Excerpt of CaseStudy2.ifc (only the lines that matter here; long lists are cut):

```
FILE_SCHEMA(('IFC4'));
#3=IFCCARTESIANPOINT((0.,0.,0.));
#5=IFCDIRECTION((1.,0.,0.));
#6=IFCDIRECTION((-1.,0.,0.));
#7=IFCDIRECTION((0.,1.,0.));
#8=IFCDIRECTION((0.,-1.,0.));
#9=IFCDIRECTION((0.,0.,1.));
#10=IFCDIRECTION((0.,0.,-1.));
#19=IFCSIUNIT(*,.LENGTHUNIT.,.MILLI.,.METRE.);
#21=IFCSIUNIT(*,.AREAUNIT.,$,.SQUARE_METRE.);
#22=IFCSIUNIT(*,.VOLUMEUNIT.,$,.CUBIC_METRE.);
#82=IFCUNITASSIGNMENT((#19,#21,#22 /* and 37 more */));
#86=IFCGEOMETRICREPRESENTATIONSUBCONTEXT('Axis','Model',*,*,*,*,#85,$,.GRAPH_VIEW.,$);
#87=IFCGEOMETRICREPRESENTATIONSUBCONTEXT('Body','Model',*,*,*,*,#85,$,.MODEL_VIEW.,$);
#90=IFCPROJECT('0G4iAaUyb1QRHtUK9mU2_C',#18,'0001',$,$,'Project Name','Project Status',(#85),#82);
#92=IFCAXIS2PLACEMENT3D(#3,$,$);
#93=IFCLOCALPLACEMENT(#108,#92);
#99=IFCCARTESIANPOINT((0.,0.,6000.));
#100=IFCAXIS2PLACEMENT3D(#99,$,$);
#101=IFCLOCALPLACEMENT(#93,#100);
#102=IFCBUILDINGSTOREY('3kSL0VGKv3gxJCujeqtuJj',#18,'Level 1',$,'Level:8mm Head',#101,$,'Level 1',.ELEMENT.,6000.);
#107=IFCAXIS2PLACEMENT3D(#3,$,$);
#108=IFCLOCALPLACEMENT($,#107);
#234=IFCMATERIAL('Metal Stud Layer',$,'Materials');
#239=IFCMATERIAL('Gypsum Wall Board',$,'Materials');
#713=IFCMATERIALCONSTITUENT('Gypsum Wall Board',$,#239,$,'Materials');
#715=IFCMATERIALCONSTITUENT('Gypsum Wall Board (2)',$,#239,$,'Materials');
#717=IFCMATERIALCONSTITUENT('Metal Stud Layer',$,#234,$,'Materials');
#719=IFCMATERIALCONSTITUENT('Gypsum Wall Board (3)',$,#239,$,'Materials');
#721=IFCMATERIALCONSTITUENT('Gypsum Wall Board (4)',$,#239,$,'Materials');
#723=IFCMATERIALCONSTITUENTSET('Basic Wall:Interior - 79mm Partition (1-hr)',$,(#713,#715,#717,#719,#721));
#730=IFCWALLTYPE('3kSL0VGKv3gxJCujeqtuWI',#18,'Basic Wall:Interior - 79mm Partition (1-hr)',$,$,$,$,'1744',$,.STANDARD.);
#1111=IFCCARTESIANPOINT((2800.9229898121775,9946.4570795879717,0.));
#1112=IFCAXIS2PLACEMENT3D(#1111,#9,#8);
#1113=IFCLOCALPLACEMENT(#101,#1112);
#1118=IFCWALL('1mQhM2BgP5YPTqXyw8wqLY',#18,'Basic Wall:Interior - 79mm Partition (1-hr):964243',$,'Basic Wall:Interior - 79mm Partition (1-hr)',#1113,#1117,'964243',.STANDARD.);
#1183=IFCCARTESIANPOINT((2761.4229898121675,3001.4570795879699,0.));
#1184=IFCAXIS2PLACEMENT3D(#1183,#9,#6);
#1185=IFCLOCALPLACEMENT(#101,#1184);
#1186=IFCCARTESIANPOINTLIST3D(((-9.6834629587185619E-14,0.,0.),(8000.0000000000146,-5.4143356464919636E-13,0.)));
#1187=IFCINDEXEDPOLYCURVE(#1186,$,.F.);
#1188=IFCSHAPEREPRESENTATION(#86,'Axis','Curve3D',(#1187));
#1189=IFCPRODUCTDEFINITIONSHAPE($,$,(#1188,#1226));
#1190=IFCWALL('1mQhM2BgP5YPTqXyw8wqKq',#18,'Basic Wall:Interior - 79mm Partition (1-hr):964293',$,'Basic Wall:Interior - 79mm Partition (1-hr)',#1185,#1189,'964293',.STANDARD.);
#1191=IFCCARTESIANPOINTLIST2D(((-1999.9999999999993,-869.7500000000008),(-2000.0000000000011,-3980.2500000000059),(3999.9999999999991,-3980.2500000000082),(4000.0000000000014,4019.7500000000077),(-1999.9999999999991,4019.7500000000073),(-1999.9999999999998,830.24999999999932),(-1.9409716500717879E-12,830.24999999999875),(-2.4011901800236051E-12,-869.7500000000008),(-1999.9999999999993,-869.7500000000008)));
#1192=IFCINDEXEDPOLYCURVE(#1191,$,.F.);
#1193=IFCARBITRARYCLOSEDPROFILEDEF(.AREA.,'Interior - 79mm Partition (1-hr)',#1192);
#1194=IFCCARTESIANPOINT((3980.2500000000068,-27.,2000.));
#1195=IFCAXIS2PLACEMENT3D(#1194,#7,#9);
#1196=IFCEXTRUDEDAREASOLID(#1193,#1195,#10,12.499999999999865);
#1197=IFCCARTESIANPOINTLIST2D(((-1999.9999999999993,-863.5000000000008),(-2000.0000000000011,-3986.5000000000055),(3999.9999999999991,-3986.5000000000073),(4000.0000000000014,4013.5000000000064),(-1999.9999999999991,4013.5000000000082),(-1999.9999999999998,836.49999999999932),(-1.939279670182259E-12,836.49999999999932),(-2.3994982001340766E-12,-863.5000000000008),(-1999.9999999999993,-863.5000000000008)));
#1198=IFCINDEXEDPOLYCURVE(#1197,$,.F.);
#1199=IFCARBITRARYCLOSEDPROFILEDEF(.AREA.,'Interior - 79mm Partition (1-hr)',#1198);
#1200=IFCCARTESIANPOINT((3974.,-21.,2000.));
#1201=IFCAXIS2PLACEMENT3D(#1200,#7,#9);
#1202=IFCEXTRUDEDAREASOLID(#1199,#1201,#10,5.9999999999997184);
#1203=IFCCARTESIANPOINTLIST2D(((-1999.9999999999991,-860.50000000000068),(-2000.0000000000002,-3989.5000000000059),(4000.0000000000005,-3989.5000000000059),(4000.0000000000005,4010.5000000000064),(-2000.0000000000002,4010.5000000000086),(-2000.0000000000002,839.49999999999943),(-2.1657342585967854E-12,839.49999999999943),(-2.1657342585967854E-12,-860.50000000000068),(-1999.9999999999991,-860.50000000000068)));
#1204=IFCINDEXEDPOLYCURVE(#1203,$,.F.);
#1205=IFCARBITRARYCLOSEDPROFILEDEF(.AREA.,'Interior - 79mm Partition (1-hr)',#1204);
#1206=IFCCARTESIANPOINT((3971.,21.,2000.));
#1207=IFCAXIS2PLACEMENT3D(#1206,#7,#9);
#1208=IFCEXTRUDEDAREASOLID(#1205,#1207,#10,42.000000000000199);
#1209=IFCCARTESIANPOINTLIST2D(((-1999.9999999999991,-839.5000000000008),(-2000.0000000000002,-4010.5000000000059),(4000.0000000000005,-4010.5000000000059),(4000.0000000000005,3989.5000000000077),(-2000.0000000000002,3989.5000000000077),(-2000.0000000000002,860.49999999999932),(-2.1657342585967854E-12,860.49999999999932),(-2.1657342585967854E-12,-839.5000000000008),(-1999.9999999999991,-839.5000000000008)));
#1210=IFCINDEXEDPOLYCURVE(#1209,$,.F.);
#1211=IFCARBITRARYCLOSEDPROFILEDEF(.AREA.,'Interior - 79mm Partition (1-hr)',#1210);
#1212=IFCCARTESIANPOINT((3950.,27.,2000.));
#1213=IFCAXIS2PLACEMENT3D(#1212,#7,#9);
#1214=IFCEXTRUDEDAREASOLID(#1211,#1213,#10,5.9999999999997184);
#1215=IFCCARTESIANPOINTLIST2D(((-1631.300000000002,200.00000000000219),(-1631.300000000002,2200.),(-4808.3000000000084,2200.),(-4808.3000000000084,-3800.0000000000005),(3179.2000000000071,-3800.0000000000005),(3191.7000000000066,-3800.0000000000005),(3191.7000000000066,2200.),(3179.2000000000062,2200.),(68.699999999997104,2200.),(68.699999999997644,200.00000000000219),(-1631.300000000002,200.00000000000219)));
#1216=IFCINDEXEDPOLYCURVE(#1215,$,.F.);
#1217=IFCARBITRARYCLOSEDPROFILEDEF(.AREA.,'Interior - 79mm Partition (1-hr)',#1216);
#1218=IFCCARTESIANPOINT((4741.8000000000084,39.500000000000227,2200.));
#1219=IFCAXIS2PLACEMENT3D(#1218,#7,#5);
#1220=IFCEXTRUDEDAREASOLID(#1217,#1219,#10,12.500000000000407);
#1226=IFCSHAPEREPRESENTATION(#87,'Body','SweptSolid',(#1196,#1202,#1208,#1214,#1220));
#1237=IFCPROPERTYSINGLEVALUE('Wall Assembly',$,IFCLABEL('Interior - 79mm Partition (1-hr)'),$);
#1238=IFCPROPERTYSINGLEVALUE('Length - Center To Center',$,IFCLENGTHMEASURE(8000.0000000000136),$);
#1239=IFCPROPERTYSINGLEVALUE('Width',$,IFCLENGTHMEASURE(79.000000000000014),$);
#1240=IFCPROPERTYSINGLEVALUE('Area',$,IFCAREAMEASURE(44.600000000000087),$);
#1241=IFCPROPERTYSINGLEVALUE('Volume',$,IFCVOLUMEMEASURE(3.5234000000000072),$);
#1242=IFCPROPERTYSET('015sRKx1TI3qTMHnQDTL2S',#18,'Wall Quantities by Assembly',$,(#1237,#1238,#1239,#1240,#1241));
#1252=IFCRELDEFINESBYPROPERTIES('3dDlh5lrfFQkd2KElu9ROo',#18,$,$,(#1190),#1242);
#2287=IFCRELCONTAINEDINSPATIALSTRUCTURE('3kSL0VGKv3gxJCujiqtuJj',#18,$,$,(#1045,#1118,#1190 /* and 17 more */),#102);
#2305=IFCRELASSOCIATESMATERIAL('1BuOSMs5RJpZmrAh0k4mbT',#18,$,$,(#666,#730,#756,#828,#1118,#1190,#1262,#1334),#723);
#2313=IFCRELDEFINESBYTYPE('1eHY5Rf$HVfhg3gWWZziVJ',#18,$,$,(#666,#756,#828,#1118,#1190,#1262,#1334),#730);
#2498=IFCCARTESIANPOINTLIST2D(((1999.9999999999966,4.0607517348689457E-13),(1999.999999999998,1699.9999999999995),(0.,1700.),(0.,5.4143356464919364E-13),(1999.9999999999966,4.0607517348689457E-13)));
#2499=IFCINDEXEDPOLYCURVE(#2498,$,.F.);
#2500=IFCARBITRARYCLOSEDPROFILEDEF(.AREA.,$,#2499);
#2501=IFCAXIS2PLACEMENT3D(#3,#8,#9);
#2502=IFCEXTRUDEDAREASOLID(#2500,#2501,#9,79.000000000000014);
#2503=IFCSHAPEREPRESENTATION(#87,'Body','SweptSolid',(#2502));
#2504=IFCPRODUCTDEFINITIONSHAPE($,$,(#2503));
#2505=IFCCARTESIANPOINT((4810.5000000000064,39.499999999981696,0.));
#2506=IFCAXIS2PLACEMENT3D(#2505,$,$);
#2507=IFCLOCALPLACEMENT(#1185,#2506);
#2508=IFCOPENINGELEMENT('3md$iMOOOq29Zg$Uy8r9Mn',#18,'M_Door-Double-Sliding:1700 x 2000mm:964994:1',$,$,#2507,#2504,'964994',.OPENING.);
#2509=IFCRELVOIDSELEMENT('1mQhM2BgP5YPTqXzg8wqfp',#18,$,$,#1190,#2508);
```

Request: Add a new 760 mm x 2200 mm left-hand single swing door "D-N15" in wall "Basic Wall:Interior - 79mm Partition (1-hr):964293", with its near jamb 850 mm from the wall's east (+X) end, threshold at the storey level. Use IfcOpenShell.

```python
import numpy as np
import ifcopenshell
import ifcopenshell.api.feature
import ifcopenshell.api.geometry
import ifcopenshell.api.pset
import ifcopenshell.api.root
import ifcopenshell.api.spatial
import ifcopenshell.geom
import ifcopenshell.util.element
import ifcopenshell.util.placement
import ifcopenshell.util.representation
import ifcopenshell.util.shape
import ifcopenshell.util.unit

model = ifcopenshell.open("CaseStudy2.ifc")
unit_scale = ifcopenshell.util.unit.calculate_unit_scale(model)
area_scale = ifcopenshell.util.unit.calculate_unit_scale(model, "AREAUNIT")
volume_scale = ifcopenshell.util.unit.calculate_unit_scale(model, "VOLUMEUNIT")
settings = ifcopenshell.geom.settings()


def volume(element):
    """Net volume in cubic metres, openings subtracted."""
    shape = ifcopenshell.geom.create_shape(settings, element)
    return ifcopenshell.util.shape.get_volume(shape.geometry)


wall = model.by_guid("1mQhM2BgP5YPTqXyw8wqKq")
storey = ifcopenshell.util.element.get_container(wall, ifc_class="IfcBuildingStorey")
context = ifcopenshell.util.representation.get_context(model, "Model", "Body", "MODEL_VIEW")
before = volume(wall)

width, height, from_end, sill = 0.76, 2.2, 0.85, 0.0  # metres

# The wall runs along its own X axis, and the end named is its -X end.
wall_shape = ifcopenshell.geom.create_shape(settings, wall)
x, y, z = ifcopenshell.util.shape.get_vertices(wall_shape.geometry).T
start = x.min() + from_end
face, thickness = float(y.min()), float(y.max() - y.min())
wall_matrix = ifcopenshell.util.placement.get_local_placement(wall.ObjectPlacement)
level = ifcopenshell.util.placement.get_local_placement(storey.ObjectPlacement)[2, 3]


def in_wall(x, y):
    """Placement at x, y metres in the wall's axes, at sill height."""
    matrix = wall_matrix.copy()
    matrix[:, 3] = wall_matrix @ np.array([x / unit_scale, y / unit_scale, 0.0, 1.0])
    matrix[2, 3] = level + sill / unit_scale
    return matrix


# Opening: a box that overshoots both wall faces by 50 mm.
opening = ifcopenshell.api.root.create_entity(model, ifc_class="IfcOpeningElement", predefined_type="OPENING")
box = ifcopenshell.api.geometry.add_wall_representation(
    model, context=context, length=width, height=height, thickness=thickness + 0.1
)
ifcopenshell.api.geometry.assign_representation(model, product=opening, representation=box)
ifcopenshell.api.geometry.edit_object_placement(model, product=opening, matrix=in_wall(start, face - 0.05), is_si=False)
ifcopenshell.api.feature.add_feature(model, feature=opening, element=wall)

door = ifcopenshell.api.root.create_entity(model, ifc_class="IfcDoor", name="D-N15", predefined_type="DOOR")
door.OverallWidth, door.OverallHeight = width / unit_scale, height / unit_scale
door.OperationType = "SINGLE_SWING_LEFT"
body = ifcopenshell.api.geometry.add_door_representation(
    model,
    context=context,
    overall_width=door.OverallWidth,
    overall_height=door.OverallHeight,
    operation_type="SINGLE_SWING_LEFT",
    lining_properties={"LiningDepth": thickness / unit_scale, "ThresholdDepth": thickness / unit_scale},
)
ifcopenshell.api.geometry.assign_representation(model, product=door, representation=body)
ifcopenshell.api.spatial.assign_container(model, products=[door], relating_structure=storey)
ifcopenshell.api.feature.add_filling(model, opening=opening, element=door)

# The lining spans the wall, so the door starts at the wall face.
ifcopenshell.api.geometry.edit_object_placement(model, product=door, matrix=in_wall(start, face), is_si=False)

after = volume(wall)

# Update the wall's stored quantities.
pset = model.by_id(ifcopenshell.util.element.get_pset(wall, "Wall Quantities by Assembly", should_inherit=False)["id"])
ifcopenshell.api.pset.edit_pset(model, pset=pset, properties={
    "Area": model.create_entity("IfcAreaMeasure", after / thickness / area_scale),
    "Volume": model.create_entity("IfcVolumeMeasure", after / volume_scale),
})

print(f"wall volume {before:.3f} -> {after:.3f} m3")

model.write("CaseStudy2_rev.ifc")
```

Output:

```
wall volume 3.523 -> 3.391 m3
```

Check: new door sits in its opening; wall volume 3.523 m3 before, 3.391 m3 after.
